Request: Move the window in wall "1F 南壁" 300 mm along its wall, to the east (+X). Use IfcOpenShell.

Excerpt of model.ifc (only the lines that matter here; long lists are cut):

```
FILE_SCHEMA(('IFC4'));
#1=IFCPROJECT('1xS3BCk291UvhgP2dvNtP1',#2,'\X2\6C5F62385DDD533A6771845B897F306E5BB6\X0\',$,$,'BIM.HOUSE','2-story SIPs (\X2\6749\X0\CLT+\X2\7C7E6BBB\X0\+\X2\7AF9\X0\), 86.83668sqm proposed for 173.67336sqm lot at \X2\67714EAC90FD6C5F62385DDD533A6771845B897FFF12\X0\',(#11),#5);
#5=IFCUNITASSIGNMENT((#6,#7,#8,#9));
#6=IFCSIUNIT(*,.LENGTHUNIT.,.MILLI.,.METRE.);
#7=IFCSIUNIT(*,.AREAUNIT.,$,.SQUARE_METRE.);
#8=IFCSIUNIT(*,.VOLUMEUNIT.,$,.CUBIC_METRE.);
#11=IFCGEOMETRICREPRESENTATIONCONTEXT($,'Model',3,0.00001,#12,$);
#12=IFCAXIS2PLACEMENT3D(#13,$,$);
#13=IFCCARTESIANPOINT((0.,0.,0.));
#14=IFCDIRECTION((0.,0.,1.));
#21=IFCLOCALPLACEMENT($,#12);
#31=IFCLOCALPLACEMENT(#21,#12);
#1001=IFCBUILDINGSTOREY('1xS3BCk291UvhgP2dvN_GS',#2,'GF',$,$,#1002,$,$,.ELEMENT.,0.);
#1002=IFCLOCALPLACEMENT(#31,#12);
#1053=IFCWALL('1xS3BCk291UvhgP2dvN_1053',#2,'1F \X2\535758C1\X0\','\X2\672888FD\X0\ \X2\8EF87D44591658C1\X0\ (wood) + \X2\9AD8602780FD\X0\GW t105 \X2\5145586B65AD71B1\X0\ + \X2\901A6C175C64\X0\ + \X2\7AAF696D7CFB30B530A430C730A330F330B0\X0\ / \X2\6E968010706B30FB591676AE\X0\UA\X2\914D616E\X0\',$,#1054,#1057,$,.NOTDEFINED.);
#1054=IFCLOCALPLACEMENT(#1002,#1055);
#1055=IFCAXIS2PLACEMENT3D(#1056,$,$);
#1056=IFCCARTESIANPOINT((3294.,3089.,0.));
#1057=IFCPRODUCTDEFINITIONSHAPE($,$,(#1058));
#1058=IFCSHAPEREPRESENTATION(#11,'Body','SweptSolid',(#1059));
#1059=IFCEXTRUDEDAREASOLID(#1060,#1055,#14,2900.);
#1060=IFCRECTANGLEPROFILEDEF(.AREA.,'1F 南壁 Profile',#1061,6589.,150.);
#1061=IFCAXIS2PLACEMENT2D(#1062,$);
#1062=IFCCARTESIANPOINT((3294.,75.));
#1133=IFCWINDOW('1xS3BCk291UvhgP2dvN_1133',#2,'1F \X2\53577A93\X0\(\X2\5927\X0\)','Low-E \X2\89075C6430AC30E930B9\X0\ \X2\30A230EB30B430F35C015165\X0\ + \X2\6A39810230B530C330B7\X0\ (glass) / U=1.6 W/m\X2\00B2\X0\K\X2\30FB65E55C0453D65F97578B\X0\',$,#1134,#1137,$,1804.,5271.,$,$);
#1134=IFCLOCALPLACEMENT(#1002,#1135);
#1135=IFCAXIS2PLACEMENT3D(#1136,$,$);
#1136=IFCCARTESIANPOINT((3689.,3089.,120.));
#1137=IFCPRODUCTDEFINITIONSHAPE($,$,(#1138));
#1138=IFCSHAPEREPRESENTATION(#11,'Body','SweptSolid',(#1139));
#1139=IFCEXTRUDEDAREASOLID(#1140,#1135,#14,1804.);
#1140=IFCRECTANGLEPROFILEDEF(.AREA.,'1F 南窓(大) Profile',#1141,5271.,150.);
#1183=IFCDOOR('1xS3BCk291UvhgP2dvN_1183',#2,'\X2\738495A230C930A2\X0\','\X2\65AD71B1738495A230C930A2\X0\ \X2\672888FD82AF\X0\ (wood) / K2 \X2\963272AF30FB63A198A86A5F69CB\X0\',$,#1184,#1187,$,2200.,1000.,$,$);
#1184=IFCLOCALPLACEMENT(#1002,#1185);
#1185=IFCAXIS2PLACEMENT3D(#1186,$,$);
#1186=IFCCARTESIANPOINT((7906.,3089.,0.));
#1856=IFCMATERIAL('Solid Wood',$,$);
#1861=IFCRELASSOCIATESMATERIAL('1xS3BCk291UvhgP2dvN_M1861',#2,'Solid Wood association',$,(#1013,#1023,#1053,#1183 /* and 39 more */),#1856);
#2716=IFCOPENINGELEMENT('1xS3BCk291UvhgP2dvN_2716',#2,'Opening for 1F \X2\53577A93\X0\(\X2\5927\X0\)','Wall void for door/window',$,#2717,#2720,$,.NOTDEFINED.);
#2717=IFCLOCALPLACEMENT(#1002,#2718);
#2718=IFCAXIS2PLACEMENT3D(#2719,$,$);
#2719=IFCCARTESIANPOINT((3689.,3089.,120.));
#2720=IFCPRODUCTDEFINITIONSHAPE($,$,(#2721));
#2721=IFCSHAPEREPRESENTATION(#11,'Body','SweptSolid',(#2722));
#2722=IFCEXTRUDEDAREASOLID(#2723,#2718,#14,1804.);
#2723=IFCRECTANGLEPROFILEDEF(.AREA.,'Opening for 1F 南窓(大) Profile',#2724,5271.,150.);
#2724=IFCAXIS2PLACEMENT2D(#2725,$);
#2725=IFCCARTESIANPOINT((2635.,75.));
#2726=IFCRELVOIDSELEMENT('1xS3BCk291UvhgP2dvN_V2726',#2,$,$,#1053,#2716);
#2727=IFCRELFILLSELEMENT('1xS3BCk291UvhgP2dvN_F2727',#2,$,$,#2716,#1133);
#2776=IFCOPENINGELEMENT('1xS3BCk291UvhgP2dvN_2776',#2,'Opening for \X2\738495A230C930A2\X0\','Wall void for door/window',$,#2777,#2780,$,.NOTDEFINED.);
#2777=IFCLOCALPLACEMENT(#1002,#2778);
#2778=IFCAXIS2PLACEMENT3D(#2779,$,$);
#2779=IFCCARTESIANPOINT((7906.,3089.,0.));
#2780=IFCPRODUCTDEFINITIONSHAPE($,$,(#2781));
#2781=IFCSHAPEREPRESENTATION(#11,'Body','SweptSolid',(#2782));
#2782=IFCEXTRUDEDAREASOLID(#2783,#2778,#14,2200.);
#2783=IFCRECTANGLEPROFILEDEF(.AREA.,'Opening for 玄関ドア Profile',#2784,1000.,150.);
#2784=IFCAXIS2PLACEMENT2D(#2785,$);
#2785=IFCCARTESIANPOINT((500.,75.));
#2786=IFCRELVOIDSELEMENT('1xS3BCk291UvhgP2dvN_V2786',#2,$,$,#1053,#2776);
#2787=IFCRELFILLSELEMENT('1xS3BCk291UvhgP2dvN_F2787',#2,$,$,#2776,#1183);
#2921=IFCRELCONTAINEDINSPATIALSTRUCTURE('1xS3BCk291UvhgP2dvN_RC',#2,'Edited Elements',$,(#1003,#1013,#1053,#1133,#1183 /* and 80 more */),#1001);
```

```python
import ifcopenshell
import ifcopenshell.api.geometry
import ifcopenshell.util.placement

model = ifcopenshell.open("model.ifc")

window = model.by_guid("1xS3BCk291UvhgP2dvN_1133")
opening = window.FillsVoids[0].RelatingOpeningElement
wall = opening.VoidsElements[0].RelatingBuildingElement

wall_matrix = ifcopenshell.util.placement.get_local_placement(wall.ObjectPlacement)
shift = wall_matrix[:3, 0] * 300.0
before = ifcopenshell.util.placement.get_local_placement(window.ObjectPlacement)[:3, 3].copy()

# The window is not placed relative to its opening, so move both.
for product in (opening, window):
    matrix = ifcopenshell.util.placement.get_local_placement(product.ObjectPlacement)
    matrix[:3, 3] += shift
    ifcopenshell.api.geometry.edit_object_placement(model, product=product, matrix=matrix, is_si=False)

after = ifcopenshell.util.placement.get_local_placement(window.ObjectPlacement)[:3, 3]
print("window moved by", (after - before).round(3) + 0.0)

model.write("model_v2.ifc")
```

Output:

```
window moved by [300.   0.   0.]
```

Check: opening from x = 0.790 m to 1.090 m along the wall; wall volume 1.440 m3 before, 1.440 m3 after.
